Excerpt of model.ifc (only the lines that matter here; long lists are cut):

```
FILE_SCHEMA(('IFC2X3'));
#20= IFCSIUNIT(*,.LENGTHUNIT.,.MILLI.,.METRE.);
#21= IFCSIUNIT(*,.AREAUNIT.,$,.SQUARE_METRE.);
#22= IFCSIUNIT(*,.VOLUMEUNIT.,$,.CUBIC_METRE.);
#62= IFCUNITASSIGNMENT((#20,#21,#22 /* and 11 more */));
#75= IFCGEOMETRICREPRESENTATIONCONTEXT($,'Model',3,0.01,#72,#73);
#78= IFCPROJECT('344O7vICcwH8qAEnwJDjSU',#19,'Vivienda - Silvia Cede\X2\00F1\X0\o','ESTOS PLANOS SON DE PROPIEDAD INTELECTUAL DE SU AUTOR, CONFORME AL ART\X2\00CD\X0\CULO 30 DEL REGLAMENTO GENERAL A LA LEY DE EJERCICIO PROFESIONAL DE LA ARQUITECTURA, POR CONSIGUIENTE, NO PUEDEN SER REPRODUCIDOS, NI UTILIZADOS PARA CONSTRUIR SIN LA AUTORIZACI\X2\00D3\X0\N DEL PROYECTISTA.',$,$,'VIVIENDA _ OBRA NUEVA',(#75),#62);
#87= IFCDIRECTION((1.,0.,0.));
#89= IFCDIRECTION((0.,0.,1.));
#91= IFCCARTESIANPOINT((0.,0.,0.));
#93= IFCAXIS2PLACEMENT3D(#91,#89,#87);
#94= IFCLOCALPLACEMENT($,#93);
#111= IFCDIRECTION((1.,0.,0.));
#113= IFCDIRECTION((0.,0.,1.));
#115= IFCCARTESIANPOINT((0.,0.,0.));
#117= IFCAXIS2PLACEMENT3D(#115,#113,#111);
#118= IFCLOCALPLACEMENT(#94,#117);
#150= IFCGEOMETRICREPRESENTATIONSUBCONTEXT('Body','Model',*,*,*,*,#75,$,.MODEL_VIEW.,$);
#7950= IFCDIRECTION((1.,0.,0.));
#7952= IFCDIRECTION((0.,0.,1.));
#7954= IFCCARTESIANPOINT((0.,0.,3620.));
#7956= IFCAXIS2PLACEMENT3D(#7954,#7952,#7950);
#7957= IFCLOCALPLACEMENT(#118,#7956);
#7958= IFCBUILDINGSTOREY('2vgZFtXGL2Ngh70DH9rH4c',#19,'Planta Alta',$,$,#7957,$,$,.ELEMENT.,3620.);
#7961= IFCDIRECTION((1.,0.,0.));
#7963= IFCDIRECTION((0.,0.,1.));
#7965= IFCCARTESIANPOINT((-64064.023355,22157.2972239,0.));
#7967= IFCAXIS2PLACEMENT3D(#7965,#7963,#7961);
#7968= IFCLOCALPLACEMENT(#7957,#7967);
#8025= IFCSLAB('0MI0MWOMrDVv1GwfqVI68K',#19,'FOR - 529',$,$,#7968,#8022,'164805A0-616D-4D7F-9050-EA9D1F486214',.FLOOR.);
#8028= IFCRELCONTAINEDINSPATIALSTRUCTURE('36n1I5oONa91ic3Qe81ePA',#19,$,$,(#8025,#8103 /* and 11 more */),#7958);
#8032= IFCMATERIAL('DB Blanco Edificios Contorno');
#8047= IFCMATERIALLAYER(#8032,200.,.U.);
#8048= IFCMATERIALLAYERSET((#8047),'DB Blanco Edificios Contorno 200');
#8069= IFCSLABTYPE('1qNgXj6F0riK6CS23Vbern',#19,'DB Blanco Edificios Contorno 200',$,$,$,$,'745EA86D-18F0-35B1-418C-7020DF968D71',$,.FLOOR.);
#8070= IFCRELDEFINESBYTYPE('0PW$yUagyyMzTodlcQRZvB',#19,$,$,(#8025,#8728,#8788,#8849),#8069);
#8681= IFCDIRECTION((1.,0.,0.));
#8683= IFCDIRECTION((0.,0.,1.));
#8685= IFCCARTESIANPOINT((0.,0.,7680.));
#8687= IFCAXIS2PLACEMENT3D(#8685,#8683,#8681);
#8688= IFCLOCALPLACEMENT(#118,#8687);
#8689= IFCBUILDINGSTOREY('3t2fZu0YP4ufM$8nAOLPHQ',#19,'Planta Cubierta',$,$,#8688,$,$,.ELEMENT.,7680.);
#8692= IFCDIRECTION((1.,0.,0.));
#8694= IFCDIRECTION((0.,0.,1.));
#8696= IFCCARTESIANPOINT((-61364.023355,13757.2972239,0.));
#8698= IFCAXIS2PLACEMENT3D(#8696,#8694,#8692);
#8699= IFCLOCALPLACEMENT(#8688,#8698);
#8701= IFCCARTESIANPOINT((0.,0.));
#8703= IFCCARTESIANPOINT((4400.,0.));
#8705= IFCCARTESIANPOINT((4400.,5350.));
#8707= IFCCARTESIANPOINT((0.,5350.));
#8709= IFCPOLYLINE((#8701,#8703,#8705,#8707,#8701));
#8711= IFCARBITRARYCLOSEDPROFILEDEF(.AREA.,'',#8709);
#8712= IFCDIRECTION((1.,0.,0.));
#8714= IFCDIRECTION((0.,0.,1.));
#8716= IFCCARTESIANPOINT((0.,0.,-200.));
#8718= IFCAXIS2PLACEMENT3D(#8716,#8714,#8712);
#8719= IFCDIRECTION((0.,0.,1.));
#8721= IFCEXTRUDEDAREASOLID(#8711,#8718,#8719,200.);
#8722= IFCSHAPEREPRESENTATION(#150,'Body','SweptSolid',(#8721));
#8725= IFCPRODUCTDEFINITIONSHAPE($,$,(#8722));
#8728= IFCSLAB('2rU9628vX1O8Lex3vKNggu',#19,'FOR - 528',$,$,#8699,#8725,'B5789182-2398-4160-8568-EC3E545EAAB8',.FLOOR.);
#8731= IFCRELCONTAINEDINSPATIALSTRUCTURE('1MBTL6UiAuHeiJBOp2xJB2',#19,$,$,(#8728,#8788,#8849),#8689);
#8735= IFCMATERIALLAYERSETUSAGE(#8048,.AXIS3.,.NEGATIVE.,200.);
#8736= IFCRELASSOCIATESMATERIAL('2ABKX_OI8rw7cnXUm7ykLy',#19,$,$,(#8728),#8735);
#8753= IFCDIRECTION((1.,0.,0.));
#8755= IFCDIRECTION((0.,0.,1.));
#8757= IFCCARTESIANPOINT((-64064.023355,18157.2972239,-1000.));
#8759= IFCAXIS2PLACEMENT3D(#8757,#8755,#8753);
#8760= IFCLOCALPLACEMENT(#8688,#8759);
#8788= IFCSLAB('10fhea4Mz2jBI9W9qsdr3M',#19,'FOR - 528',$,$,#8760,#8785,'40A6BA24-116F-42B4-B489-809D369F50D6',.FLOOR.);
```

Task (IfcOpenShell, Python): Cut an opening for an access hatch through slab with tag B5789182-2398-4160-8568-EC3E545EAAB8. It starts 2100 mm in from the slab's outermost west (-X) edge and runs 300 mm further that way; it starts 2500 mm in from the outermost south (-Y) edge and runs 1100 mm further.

```python
import numpy as np
import ifcopenshell
import ifcopenshell.api.feature
import ifcopenshell.api.geometry
import ifcopenshell.api.root
import ifcopenshell.geom
import ifcopenshell.util.placement
import ifcopenshell.util.representation
import ifcopenshell.util.shape
import ifcopenshell.util.unit

model = ifcopenshell.open("model.ifc")
unit_scale = ifcopenshell.util.unit.calculate_unit_scale(model)
settings = ifcopenshell.geom.settings()


def volume(element):
    """Net volume in cubic metres, openings subtracted."""
    shape = ifcopenshell.geom.create_shape(settings, element)
    return ifcopenshell.util.shape.get_volume(shape.geometry)


slab = model.by_guid("2rU9628vX1O8Lex3vKNggu")
before = volume(slab)

# Extent in the slab's own axes, in metres. The edges named are its -X and -Y sides.
slab_shape = ifcopenshell.geom.create_shape(settings, slab)
vertices = ifcopenshell.util.shape.get_vertices(slab_shape.geometry)
x_min, y_min, bottom = vertices.min(axis=0)
top = vertices[:, 2].max()

opening = ifcopenshell.api.root.create_entity(model, ifc_class="IfcOpeningElement", name="Access hatch opening")
context = ifcopenshell.util.representation.get_context(model, "Model", "Body", "MODEL_VIEW")
width, depth = 0.3, 1.1
outline = [(0.0, 0.0), (width, 0.0), (width, depth), (0.0, depth), (0.0, 0.0)]
# Overshoot both faces by 50 mm so the cut is clean.
shape = ifcopenshell.api.geometry.add_slab_representation(
    model, context=context, depth=top - bottom + 0.1, polyline=outline
)
ifcopenshell.api.geometry.assign_representation(model, product=opening, representation=shape)

matrix = ifcopenshell.util.placement.get_local_placement(slab.ObjectPlacement)
matrix[:, 3] = matrix @ np.append(np.array([x_min + 2.1, y_min + 2.5, bottom - 0.05]) / unit_scale, 1.0)
ifcopenshell.api.geometry.edit_object_placement(model, product=opening, matrix=matrix, is_si=False)
ifcopenshell.api.feature.add_feature(model, feature=opening, element=slab)

after = volume(slab)

print(f"slab volume {before:.3f} -> {after:.3f} m3")

model.write("model_updated.ifc")
```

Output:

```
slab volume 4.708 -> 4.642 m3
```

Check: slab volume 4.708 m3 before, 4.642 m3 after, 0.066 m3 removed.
